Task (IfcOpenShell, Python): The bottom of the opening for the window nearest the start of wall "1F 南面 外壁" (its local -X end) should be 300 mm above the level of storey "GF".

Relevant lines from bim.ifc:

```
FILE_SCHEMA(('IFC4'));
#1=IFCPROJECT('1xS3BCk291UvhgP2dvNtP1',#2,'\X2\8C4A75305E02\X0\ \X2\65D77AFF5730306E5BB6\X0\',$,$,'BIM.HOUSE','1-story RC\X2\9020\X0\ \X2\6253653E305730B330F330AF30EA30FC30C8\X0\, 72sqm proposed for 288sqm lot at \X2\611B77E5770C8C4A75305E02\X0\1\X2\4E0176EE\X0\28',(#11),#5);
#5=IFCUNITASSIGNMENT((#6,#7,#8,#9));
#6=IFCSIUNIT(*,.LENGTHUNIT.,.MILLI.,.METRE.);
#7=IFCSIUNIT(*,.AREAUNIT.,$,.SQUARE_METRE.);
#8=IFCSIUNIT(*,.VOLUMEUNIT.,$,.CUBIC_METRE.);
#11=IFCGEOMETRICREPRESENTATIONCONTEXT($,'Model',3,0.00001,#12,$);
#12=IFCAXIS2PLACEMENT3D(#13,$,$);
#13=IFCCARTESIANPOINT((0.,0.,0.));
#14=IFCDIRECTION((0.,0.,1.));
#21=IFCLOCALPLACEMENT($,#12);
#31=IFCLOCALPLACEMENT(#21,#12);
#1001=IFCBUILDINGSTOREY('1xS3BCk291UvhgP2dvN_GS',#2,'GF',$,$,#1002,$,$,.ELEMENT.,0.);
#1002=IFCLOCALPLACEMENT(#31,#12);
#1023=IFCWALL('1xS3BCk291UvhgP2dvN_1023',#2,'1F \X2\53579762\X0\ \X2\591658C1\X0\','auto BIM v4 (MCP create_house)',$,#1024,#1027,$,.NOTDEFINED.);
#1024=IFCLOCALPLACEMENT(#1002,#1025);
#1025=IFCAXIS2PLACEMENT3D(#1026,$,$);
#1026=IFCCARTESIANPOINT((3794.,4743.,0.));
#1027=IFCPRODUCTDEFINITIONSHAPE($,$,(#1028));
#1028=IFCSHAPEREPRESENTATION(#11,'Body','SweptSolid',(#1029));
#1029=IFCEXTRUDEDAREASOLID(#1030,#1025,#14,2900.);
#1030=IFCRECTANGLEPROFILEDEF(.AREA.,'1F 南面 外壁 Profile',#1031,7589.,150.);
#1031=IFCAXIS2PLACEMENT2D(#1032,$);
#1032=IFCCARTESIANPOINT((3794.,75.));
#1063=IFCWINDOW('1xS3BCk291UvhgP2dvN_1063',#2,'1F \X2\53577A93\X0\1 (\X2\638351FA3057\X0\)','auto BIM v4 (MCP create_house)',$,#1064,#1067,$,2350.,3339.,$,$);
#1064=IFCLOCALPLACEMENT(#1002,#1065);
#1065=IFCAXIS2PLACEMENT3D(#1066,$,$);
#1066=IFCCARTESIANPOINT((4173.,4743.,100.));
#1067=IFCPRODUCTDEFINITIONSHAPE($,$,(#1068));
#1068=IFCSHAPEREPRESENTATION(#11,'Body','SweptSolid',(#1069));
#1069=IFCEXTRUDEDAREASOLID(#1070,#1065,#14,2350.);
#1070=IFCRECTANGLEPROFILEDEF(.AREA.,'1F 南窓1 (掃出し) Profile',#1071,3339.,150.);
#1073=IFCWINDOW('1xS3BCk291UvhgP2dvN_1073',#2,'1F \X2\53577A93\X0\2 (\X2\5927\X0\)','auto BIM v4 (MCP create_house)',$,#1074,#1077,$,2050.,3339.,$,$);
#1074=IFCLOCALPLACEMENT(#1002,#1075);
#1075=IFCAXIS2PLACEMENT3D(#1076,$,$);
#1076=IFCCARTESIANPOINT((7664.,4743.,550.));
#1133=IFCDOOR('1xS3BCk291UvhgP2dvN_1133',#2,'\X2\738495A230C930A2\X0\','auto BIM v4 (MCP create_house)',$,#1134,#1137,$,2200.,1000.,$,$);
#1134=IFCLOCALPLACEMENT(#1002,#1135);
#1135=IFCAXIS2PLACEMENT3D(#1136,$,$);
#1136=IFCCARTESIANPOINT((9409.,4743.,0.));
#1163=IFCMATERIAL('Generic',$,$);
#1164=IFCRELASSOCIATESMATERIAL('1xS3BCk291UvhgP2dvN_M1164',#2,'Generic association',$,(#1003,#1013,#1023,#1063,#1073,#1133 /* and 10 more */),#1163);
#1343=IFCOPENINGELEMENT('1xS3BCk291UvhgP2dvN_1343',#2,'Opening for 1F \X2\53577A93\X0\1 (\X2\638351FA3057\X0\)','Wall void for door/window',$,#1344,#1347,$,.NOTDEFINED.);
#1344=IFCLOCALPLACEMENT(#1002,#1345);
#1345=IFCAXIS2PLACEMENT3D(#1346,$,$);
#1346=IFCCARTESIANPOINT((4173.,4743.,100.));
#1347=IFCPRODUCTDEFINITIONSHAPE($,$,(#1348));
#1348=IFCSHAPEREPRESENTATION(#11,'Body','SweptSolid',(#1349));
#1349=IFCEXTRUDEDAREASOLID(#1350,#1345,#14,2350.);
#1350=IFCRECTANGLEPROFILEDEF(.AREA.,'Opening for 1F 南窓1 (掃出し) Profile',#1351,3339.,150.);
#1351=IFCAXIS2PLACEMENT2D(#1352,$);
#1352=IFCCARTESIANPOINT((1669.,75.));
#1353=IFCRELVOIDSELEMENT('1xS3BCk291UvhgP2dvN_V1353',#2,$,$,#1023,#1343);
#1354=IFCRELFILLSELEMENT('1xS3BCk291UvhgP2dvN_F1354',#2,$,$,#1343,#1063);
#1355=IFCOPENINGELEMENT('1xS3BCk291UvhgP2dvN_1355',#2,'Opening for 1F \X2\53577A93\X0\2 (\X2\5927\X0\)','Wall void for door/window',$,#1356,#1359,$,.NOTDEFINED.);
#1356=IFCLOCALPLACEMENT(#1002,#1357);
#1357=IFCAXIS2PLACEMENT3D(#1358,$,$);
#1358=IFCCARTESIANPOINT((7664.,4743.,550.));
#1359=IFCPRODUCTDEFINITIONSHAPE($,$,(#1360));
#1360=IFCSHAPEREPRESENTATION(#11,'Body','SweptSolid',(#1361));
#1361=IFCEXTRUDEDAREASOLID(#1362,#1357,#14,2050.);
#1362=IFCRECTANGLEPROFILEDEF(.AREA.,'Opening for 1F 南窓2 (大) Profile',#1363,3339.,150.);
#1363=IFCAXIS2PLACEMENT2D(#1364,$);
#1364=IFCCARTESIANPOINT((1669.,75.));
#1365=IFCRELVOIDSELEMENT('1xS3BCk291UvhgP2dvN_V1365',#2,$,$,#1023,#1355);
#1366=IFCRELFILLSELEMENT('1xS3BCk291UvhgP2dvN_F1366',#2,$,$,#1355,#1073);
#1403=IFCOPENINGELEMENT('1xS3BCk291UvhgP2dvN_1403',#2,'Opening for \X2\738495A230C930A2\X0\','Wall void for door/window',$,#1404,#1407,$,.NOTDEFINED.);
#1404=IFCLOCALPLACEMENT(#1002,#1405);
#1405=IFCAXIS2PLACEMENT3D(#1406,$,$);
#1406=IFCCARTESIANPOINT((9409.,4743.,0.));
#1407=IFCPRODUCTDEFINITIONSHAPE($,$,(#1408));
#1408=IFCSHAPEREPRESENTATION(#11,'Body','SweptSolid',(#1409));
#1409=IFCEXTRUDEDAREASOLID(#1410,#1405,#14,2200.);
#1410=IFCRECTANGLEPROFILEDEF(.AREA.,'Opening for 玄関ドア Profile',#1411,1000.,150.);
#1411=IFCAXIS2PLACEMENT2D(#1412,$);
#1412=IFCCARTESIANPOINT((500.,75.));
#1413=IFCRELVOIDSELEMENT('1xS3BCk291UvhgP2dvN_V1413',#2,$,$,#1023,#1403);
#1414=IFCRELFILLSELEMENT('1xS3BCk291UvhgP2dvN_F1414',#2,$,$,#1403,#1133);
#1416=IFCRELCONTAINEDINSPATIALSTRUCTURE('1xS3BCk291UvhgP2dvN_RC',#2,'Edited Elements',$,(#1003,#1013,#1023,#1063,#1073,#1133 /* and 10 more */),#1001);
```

```python
import numpy as np
import ifcopenshell
import ifcopenshell.api.geometry
import ifcopenshell.geom
import ifcopenshell.util.element
import ifcopenshell.util.placement
import ifcopenshell.util.shape
import ifcopenshell.util.unit

model = ifcopenshell.open("bim.ifc")
unit_scale = ifcopenshell.util.unit.calculate_unit_scale(model)

window = model.by_guid("1xS3BCk291UvhgP2dvN_1063")
opening = window.FillsVoids[0].RelatingOpeningElement
storey = ifcopenshell.util.element.get_container(window, ifc_class="IfcBuildingStorey")
level = ifcopenshell.util.placement.get_local_placement(storey.ObjectPlacement)[2, 3]

# The opening's origin need not be at the sill, so measure its lowest point.
shape = ifcopenshell.geom.create_shape(ifcopenshell.geom.settings(), opening)
bottom = ifcopenshell.util.shape.get_shape_bottom_elevation(shape, shape.geometry) / unit_scale
dz = level + 0.3 / unit_scale - bottom

shift = np.array([0.0, 0.0, dz])
# The window is not placed relative to its opening, so move both.
for product in (opening, window):
    matrix = ifcopenshell.util.placement.get_local_placement(product.ObjectPlacement)
    matrix[:3, 3] += shift
    ifcopenshell.api.geometry.edit_object_placement(model, product=product, matrix=matrix, is_si=False)

print(f"moved by {dz * unit_scale:+.3f} m")

model.write("bim-out.ifc")
```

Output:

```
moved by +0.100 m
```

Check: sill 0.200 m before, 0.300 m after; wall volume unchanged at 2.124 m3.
